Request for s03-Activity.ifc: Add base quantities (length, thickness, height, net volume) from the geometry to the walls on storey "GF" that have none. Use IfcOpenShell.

First a look at what the model holds.

```python
import ifcopenshell
import ifcopenshell.util.element
import ifcopenshell.util.unit

model = ifcopenshell.open("s03-Activity.ifc")
print(model.schema)
for unit_type in ("LENGTHUNIT", "AREAUNIT", "VOLUMEUNIT"):
    print(unit_type, ifcopenshell.util.unit.calculate_unit_scale(model, unit_type))
storey = next(s for s in model.by_type("IfcBuildingStorey") if s.Name == "GF")
walls = [e for e in ifcopenshell.util.element.get_decomposition(storey) if e.is_a("IfcWall")]
for e in sorted(walls, key=lambda e: e.id()):
    print(e.id(), e.is_a(), e.Name, list(ifcopenshell.util.element.get_psets(e, qtos_only=True)), sep=" | ")
```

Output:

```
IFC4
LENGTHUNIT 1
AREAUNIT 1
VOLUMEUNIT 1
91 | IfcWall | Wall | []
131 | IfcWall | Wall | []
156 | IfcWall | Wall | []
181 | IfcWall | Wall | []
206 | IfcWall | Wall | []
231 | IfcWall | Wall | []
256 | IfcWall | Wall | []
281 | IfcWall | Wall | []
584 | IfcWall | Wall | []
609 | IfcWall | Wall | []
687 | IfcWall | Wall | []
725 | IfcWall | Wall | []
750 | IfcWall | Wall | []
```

```python
import ifcopenshell
import ifcopenshell.api.pset
import ifcopenshell.geom
import ifcopenshell.util.element
import ifcopenshell.util.shape
import ifcopenshell.util.unit

model = ifcopenshell.open("s03-Activity.ifc")
unit_scale = ifcopenshell.util.unit.calculate_unit_scale(model)
volume_scale = ifcopenshell.util.unit.calculate_unit_scale(model, "VOLUMEUNIT")
settings = ifcopenshell.geom.settings()

storey = next(s for s in model.by_type("IfcBuildingStorey") if s.Name == "GF")
walls = [e for e in ifcopenshell.util.element.get_decomposition(storey) if e.is_a("IfcWall")]

for e in sorted(walls, key=lambda e: e.id()):
    if ifcopenshell.util.element.get_psets(e, qtos_only=True, should_inherit=False):
        continue
    # Geometry comes back in metres, in the element's own axes.
    shape = ifcopenshell.geom.create_shape(settings, e)
    values = {
        "Length": ifcopenshell.util.shape.get_x(shape.geometry) / unit_scale,
        "Width": ifcopenshell.util.shape.get_y(shape.geometry) / unit_scale,
        "Height": ifcopenshell.util.shape.get_z(shape.geometry) / unit_scale,
        "NetVolume": ifcopenshell.util.shape.get_volume(shape.geometry) / volume_scale,
    }
    qto = ifcopenshell.api.pset.add_qto(model, product=e, name="Qto_WallBaseQuantities")
    ifcopenshell.api.pset.edit_qto(model, qto=qto, properties=values)
    print(e.id(), {k: round(v, 3) for k, v in values.items()})

model.write("s03-Activity-out.ifc")
```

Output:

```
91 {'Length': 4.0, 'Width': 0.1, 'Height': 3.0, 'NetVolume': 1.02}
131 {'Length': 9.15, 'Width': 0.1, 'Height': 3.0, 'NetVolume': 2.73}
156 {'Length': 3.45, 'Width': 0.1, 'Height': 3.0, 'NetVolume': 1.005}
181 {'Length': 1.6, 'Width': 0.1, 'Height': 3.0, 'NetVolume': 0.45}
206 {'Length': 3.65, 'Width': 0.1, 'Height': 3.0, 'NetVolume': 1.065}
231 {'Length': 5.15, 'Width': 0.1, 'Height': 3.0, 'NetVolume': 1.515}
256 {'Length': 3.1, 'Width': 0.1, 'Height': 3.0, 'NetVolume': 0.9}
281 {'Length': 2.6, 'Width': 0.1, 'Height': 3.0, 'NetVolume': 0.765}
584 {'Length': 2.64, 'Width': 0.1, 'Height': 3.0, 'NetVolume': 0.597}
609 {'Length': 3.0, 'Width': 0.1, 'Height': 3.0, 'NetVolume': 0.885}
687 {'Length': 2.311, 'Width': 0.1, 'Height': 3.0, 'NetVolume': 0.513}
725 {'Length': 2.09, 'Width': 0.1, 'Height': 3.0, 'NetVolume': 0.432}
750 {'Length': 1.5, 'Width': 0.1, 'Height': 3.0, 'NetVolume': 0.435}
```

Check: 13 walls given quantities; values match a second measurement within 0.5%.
